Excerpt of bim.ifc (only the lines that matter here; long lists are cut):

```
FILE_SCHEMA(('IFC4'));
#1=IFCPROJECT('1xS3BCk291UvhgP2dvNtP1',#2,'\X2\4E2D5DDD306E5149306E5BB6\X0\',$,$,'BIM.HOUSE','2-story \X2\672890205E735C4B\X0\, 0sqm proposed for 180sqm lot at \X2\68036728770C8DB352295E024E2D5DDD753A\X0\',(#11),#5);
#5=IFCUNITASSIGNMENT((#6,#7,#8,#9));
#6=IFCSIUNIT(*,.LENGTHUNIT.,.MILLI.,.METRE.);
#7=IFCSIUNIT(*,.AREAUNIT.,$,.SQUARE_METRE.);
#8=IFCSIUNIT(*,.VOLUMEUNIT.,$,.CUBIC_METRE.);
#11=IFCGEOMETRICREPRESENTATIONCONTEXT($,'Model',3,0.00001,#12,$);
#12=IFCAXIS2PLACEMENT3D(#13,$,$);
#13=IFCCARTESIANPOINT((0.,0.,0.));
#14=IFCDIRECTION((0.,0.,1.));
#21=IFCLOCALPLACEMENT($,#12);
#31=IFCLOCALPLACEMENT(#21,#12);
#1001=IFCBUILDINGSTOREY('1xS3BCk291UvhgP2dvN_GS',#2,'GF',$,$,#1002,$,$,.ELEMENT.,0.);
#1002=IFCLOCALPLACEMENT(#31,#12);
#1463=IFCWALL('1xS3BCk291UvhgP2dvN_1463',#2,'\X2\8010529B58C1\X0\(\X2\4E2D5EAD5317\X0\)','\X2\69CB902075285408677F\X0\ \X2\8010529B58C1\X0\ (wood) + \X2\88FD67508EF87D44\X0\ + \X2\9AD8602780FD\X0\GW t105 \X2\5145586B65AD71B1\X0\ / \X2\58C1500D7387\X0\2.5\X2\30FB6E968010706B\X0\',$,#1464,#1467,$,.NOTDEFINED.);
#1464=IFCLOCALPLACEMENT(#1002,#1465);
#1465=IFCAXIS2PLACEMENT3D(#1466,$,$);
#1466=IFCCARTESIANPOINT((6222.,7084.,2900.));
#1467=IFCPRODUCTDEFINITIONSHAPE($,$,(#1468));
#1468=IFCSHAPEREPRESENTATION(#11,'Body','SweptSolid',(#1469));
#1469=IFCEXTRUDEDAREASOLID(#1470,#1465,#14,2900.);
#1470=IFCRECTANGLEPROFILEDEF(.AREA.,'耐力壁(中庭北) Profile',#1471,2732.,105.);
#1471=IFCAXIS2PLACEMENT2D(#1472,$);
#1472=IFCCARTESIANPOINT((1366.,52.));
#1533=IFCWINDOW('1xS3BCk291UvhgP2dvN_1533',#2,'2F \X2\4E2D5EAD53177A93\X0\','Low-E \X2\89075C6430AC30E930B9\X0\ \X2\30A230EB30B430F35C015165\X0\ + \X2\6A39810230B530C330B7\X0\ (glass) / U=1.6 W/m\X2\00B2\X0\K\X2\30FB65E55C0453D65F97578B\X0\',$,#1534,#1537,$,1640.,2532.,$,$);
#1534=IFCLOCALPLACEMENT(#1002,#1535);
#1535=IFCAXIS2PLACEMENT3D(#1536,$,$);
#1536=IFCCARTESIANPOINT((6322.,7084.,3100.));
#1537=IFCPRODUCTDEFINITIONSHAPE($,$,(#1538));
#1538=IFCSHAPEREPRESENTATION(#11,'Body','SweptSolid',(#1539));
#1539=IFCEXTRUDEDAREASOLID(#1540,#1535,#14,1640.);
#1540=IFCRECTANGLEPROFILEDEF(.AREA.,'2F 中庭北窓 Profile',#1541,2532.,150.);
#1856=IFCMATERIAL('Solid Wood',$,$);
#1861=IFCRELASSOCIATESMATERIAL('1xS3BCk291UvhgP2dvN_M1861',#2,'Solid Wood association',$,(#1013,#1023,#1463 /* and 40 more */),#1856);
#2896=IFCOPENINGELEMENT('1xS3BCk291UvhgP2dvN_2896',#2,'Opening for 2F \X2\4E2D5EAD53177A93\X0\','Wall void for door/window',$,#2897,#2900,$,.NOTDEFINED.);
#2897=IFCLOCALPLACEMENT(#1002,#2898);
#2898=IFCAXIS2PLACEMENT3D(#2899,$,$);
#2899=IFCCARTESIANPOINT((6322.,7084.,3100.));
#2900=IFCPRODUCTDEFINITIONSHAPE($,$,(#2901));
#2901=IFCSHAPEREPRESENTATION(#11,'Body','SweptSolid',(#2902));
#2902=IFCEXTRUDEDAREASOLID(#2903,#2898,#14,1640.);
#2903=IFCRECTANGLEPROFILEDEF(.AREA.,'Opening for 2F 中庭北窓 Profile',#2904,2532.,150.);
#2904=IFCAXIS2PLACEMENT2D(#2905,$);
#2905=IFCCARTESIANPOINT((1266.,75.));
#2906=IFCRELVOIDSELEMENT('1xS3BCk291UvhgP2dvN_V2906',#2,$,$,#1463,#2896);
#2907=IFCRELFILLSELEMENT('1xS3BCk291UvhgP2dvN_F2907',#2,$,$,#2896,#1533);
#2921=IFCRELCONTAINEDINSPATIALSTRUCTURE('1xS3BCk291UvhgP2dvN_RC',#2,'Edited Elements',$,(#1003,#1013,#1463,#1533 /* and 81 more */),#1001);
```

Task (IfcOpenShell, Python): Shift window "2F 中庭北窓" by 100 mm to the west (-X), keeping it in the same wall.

```python
import ifcopenshell
import ifcopenshell.api.geometry
import ifcopenshell.util.placement
import ifcopenshell.util.unit

model = ifcopenshell.open("bim.ifc")
unit_scale = ifcopenshell.util.unit.calculate_unit_scale(model)

window = model.by_guid("1xS3BCk291UvhgP2dvN_1533")
opening = window.FillsVoids[0].RelatingOpeningElement
wall = opening.VoidsElements[0].RelatingBuildingElement

wall_matrix = ifcopenshell.util.placement.get_local_placement(wall.ObjectPlacement)
shift = wall_matrix[:3, 0] * -0.1 / unit_scale
before = ifcopenshell.util.placement.get_local_placement(window.ObjectPlacement)[:3, 3].copy()

# The window is not placed relative to its opening, so move both.
for product in (opening, window):
    matrix = ifcopenshell.util.placement.get_local_placement(product.ObjectPlacement)
    matrix[:3, 3] += shift
    ifcopenshell.api.geometry.edit_object_placement(model, product=product, matrix=matrix, is_si=False)

after = ifcopenshell.util.placement.get_local_placement(window.ObjectPlacement)[:3, 3]
print("window moved by", (after - before).round(3) + 0.0)

model.write("bim_v2.ifc")
```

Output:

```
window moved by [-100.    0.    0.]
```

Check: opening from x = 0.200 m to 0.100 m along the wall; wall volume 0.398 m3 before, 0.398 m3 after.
